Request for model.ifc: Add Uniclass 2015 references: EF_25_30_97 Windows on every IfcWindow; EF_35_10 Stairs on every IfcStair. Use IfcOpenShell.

First a look at what the model holds.

```python
import ifcopenshell

model = ifcopenshell.open("model.ifc")
print(model.schema)
print("classifications:", [c.Name for c in model.by_type("IfcClassification")])
for ifc_class in ("IfcDoor", "IfcRoof", "IfcStair", "IfcWall", "IfcWindow"):
    print(ifc_class, len(model.by_type(ifc_class)))
```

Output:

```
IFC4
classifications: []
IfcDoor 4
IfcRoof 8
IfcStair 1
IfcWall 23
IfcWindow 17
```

```python
import ifcopenshell
import ifcopenshell.api.classification

model = ifcopenshell.open("model.ifc")

system = ifcopenshell.api.classification.add_classification(model, classification="Uniclass 2015")

codes = {
    "IfcWindow": ("EF_25_30_97", "Windows"),
    "IfcStair": ("EF_35_10", "Stairs"),
}
for ifc_class, (code, name) in codes.items():
    products = model.by_type(ifc_class)
    ifcopenshell.api.classification.add_reference(
        model, products=products, classification=system, identification=code, name=name
    )
    print(code, len(products))

model.write("model_edited.ifc")
```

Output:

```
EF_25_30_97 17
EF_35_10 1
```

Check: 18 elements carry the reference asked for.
